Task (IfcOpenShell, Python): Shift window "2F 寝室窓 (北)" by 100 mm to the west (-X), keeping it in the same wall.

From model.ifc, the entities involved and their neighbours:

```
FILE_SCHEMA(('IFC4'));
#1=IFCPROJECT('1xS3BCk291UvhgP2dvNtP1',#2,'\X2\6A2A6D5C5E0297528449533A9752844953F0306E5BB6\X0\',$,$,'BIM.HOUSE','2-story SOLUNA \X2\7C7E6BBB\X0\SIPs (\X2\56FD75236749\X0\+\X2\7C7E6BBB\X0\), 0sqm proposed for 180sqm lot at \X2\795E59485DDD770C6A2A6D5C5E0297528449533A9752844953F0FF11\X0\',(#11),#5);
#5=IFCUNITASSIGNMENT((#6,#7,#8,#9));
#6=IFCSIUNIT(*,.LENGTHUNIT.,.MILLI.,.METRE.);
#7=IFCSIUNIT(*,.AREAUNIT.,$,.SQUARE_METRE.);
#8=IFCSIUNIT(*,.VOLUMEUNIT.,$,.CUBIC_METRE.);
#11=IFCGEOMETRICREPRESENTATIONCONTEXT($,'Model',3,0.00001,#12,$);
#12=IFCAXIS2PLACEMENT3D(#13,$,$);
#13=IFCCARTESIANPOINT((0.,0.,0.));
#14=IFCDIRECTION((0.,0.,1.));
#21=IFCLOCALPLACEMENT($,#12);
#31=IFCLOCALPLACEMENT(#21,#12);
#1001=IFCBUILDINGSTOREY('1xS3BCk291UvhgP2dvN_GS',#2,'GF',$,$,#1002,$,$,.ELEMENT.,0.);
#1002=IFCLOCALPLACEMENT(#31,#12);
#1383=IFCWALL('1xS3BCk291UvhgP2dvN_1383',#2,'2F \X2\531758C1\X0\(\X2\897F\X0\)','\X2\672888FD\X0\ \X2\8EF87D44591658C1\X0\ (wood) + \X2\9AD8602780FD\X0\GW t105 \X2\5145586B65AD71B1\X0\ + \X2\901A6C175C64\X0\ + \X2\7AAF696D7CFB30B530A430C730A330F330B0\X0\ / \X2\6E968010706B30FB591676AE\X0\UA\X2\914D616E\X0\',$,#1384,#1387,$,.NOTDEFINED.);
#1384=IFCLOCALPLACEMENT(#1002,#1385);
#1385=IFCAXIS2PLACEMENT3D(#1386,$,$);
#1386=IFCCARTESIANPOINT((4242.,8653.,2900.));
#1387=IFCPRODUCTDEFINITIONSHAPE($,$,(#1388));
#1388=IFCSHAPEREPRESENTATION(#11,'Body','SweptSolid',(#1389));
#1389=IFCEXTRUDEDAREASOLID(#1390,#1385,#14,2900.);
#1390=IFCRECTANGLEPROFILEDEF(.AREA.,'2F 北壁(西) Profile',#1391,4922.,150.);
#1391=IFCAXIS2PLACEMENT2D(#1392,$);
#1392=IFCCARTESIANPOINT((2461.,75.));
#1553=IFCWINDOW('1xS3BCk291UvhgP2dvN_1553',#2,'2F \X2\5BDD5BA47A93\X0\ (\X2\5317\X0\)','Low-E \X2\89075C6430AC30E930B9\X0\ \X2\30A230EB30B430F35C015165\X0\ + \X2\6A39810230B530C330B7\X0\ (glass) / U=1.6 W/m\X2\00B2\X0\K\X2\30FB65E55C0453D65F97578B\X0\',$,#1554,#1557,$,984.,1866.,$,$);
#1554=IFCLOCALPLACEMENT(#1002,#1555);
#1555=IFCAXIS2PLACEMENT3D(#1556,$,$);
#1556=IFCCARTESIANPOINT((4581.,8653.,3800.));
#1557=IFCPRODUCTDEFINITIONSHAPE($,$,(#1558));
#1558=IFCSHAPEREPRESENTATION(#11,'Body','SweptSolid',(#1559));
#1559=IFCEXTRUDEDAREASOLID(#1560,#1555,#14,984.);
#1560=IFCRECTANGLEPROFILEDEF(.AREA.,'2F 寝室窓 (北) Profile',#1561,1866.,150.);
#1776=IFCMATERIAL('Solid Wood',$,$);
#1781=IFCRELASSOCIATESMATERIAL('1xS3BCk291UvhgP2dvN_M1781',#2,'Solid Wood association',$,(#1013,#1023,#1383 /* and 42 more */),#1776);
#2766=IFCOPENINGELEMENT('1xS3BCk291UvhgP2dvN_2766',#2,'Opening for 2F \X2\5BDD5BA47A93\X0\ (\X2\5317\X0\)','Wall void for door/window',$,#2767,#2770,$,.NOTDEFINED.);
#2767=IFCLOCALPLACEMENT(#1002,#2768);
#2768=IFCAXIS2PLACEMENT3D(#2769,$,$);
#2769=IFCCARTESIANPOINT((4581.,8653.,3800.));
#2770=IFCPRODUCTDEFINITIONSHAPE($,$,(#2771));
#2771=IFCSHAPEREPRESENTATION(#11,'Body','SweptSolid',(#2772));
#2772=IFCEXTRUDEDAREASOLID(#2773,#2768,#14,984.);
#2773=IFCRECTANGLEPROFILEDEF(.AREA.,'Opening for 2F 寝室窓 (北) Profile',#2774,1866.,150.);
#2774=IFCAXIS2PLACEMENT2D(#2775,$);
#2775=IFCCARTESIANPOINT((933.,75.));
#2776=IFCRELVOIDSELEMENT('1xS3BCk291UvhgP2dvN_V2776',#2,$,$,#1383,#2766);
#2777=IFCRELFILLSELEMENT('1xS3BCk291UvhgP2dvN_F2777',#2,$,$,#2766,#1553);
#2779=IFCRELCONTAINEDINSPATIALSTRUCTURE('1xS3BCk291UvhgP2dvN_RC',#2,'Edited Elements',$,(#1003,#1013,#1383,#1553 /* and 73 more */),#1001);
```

```python
import ifcopenshell
import ifcopenshell.api.geometry
import ifcopenshell.util.placement
import ifcopenshell.util.unit

model = ifcopenshell.open("model.ifc")
unit_scale = ifcopenshell.util.unit.calculate_unit_scale(model)

window = model.by_guid("1xS3BCk291UvhgP2dvN_1553")
opening = window.FillsVoids[0].RelatingOpeningElement
wall = opening.VoidsElements[0].RelatingBuildingElement

wall_matrix = ifcopenshell.util.placement.get_local_placement(wall.ObjectPlacement)
shift = wall_matrix[:3, 0] * -0.1 / unit_scale
before = ifcopenshell.util.placement.get_local_placement(window.ObjectPlacement)[:3, 3].copy()

# The window is not placed relative to its opening, so move both.
for product in (opening, window):
    matrix = ifcopenshell.util.placement.get_local_placement(product.ObjectPlacement)
    matrix[:3, 3] += shift
    ifcopenshell.api.geometry.edit_object_placement(model, product=product, matrix=matrix, is_si=False)

after = ifcopenshell.util.placement.get_local_placement(window.ObjectPlacement)[:3, 3]
print("window moved by", (after - before).round(3) + 0.0)

model.write("model-out.ifc")
```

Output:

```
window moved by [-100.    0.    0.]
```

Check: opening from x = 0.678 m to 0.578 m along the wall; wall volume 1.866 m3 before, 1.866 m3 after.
